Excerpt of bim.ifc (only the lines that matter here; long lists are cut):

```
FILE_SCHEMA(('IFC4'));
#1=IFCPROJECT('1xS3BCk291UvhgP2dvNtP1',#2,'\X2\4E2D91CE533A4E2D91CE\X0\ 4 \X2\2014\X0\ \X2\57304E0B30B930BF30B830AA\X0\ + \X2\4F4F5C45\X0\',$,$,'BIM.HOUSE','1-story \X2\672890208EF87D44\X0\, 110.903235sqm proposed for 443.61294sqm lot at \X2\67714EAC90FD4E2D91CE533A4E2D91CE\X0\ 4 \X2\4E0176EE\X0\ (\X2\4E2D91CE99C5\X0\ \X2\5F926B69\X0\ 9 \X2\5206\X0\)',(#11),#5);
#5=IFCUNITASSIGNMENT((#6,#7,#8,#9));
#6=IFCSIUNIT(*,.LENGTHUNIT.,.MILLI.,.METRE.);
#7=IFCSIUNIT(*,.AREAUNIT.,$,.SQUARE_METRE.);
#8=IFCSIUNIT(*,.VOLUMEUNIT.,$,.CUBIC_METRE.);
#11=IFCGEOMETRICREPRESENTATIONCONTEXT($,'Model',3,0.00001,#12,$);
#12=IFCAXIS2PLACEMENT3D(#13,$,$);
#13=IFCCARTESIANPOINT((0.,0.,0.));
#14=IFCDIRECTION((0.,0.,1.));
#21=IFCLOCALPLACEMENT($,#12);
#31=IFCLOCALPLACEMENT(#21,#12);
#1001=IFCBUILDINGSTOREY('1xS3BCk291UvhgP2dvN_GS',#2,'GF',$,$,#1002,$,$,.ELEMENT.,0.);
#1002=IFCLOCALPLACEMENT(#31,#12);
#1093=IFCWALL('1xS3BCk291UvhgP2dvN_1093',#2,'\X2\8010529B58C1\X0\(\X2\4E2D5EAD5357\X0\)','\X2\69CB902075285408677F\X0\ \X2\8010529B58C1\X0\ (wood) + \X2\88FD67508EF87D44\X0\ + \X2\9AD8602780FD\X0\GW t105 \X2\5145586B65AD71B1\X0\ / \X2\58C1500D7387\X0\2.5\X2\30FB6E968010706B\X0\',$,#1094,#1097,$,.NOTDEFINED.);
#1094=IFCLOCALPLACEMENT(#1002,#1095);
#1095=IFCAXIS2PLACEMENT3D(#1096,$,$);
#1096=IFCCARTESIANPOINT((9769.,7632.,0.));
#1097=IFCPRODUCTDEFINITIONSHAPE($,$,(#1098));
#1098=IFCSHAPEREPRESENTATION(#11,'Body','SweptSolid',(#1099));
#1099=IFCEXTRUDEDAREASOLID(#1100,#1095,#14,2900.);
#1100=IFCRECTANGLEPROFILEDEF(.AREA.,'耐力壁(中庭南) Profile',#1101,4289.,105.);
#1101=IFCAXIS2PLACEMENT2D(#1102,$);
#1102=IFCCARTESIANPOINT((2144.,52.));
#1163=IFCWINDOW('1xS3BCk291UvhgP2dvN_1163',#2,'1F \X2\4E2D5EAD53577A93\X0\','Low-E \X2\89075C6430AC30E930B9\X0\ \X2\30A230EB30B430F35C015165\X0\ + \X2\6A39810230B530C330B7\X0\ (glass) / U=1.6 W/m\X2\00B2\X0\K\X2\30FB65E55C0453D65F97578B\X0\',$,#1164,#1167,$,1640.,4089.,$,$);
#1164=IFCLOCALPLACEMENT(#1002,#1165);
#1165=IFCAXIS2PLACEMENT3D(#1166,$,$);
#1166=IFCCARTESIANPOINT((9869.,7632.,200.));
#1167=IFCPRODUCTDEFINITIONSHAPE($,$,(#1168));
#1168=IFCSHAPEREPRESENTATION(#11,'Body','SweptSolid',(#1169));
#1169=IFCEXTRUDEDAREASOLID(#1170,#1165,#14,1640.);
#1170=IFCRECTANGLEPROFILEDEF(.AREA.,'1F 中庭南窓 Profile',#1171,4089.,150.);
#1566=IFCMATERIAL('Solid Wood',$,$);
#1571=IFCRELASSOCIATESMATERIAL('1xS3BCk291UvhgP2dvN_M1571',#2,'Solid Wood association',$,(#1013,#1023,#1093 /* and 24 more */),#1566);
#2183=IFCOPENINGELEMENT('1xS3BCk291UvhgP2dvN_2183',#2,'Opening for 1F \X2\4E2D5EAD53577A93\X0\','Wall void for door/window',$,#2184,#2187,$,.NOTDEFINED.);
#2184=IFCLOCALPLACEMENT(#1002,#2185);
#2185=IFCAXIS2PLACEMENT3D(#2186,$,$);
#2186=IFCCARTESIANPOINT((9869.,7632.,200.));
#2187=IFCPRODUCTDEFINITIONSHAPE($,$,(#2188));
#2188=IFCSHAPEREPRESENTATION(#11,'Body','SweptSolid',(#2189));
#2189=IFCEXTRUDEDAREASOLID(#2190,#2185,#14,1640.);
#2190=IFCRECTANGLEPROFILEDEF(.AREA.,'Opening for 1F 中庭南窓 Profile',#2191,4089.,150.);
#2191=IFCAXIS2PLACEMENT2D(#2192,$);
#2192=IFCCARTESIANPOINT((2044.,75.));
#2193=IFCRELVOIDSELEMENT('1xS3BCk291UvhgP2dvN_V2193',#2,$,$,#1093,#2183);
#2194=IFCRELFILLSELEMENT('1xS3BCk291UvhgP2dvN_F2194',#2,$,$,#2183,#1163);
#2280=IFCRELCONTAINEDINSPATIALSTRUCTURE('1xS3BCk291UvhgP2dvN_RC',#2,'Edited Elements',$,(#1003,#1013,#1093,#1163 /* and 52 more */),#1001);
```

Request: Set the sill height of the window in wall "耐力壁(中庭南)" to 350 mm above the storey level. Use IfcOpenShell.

```python
import numpy as np
import ifcopenshell
import ifcopenshell.api.geometry
import ifcopenshell.geom
import ifcopenshell.util.element
import ifcopenshell.util.placement
import ifcopenshell.util.shape
import ifcopenshell.util.unit

model = ifcopenshell.open("bim.ifc")
unit_scale = ifcopenshell.util.unit.calculate_unit_scale(model)

window = model.by_guid("1xS3BCk291UvhgP2dvN_1163")
opening = window.FillsVoids[0].RelatingOpeningElement
storey = ifcopenshell.util.element.get_container(window, ifc_class="IfcBuildingStorey")
level = ifcopenshell.util.placement.get_local_placement(storey.ObjectPlacement)[2, 3]

# The opening's origin need not be at the sill, so measure its lowest point.
shape = ifcopenshell.geom.create_shape(ifcopenshell.geom.settings(), opening)
bottom = ifcopenshell.util.shape.get_shape_bottom_elevation(shape, shape.geometry) / unit_scale
dz = level + 0.35 / unit_scale - bottom

shift = np.array([0.0, 0.0, dz])
# The window is not placed relative to its opening, so move both.
for product in (opening, window):
    matrix = ifcopenshell.util.placement.get_local_placement(product.ObjectPlacement)
    matrix[:3, 3] += shift
    ifcopenshell.api.geometry.edit_object_placement(model, product=product, matrix=matrix, is_si=False)

print(f"moved by {dz * unit_scale:+.3f} m")

model.write("bim_edited.ifc")
```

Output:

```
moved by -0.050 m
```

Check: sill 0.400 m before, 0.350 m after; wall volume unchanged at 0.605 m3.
